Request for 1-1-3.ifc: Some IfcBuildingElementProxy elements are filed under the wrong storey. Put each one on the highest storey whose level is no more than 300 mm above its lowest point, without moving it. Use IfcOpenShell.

First a look at what the model holds.

```python
import ifcopenshell
import ifcopenshell.util.element
import ifcopenshell.util.placement

model = ifcopenshell.open("1-1-3.ifc")
print(model.schema)
for storey in model.by_type("IfcBuildingStorey"):
    level = ifcopenshell.util.placement.get_storey_elevation(storey)
    count = sum(e.is_a("IfcBuildingElementProxy") for e in ifcopenshell.util.element.get_contained(storey))
    print(storey.id(), storey.Name, round(level, 3), count, sep=" | ")
```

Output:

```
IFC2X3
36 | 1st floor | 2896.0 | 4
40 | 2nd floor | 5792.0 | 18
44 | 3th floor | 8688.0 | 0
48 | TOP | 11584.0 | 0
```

```python
import ifcopenshell
import ifcopenshell.api.spatial
import ifcopenshell.geom
import ifcopenshell.util.element
import ifcopenshell.util.placement
import ifcopenshell.util.shape
import ifcopenshell.util.unit

model = ifcopenshell.open("1-1-3.ifc")
unit_scale = ifcopenshell.util.unit.calculate_unit_scale(model)
settings = ifcopenshell.geom.settings()

levels = sorted(
    ((ifcopenshell.util.placement.get_storey_elevation(s) * unit_scale, s) for s in model.by_type("IfcBuildingStorey")),
    key=lambda pair: pair[0],
)

for e in model.by_type("IfcBuildingElementProxy"):
    current = e.ContainedInStructure[0].RelatingStructure if e.ContainedInStructure else None
    if current is None or not current.is_a("IfcBuildingStorey"):
        continue
    shape = ifcopenshell.geom.create_shape(settings, e)
    bottom = ifcopenshell.util.shape.get_shape_bottom_elevation(shape, shape.geometry)
    below = [s for level, s in levels if level <= bottom + 0.3]
    storey = below[-1] if below else levels[0][1]
    if storey != current:
        # assign_container keeps the world position.
        ifcopenshell.api.spatial.assign_container(model, products=[e], relating_structure=storey)
        print(e.id(), current.Name, "->", storey.Name)

model.write("1-1-3-out.ifc")
```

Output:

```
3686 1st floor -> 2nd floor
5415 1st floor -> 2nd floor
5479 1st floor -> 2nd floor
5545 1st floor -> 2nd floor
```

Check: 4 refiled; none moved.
